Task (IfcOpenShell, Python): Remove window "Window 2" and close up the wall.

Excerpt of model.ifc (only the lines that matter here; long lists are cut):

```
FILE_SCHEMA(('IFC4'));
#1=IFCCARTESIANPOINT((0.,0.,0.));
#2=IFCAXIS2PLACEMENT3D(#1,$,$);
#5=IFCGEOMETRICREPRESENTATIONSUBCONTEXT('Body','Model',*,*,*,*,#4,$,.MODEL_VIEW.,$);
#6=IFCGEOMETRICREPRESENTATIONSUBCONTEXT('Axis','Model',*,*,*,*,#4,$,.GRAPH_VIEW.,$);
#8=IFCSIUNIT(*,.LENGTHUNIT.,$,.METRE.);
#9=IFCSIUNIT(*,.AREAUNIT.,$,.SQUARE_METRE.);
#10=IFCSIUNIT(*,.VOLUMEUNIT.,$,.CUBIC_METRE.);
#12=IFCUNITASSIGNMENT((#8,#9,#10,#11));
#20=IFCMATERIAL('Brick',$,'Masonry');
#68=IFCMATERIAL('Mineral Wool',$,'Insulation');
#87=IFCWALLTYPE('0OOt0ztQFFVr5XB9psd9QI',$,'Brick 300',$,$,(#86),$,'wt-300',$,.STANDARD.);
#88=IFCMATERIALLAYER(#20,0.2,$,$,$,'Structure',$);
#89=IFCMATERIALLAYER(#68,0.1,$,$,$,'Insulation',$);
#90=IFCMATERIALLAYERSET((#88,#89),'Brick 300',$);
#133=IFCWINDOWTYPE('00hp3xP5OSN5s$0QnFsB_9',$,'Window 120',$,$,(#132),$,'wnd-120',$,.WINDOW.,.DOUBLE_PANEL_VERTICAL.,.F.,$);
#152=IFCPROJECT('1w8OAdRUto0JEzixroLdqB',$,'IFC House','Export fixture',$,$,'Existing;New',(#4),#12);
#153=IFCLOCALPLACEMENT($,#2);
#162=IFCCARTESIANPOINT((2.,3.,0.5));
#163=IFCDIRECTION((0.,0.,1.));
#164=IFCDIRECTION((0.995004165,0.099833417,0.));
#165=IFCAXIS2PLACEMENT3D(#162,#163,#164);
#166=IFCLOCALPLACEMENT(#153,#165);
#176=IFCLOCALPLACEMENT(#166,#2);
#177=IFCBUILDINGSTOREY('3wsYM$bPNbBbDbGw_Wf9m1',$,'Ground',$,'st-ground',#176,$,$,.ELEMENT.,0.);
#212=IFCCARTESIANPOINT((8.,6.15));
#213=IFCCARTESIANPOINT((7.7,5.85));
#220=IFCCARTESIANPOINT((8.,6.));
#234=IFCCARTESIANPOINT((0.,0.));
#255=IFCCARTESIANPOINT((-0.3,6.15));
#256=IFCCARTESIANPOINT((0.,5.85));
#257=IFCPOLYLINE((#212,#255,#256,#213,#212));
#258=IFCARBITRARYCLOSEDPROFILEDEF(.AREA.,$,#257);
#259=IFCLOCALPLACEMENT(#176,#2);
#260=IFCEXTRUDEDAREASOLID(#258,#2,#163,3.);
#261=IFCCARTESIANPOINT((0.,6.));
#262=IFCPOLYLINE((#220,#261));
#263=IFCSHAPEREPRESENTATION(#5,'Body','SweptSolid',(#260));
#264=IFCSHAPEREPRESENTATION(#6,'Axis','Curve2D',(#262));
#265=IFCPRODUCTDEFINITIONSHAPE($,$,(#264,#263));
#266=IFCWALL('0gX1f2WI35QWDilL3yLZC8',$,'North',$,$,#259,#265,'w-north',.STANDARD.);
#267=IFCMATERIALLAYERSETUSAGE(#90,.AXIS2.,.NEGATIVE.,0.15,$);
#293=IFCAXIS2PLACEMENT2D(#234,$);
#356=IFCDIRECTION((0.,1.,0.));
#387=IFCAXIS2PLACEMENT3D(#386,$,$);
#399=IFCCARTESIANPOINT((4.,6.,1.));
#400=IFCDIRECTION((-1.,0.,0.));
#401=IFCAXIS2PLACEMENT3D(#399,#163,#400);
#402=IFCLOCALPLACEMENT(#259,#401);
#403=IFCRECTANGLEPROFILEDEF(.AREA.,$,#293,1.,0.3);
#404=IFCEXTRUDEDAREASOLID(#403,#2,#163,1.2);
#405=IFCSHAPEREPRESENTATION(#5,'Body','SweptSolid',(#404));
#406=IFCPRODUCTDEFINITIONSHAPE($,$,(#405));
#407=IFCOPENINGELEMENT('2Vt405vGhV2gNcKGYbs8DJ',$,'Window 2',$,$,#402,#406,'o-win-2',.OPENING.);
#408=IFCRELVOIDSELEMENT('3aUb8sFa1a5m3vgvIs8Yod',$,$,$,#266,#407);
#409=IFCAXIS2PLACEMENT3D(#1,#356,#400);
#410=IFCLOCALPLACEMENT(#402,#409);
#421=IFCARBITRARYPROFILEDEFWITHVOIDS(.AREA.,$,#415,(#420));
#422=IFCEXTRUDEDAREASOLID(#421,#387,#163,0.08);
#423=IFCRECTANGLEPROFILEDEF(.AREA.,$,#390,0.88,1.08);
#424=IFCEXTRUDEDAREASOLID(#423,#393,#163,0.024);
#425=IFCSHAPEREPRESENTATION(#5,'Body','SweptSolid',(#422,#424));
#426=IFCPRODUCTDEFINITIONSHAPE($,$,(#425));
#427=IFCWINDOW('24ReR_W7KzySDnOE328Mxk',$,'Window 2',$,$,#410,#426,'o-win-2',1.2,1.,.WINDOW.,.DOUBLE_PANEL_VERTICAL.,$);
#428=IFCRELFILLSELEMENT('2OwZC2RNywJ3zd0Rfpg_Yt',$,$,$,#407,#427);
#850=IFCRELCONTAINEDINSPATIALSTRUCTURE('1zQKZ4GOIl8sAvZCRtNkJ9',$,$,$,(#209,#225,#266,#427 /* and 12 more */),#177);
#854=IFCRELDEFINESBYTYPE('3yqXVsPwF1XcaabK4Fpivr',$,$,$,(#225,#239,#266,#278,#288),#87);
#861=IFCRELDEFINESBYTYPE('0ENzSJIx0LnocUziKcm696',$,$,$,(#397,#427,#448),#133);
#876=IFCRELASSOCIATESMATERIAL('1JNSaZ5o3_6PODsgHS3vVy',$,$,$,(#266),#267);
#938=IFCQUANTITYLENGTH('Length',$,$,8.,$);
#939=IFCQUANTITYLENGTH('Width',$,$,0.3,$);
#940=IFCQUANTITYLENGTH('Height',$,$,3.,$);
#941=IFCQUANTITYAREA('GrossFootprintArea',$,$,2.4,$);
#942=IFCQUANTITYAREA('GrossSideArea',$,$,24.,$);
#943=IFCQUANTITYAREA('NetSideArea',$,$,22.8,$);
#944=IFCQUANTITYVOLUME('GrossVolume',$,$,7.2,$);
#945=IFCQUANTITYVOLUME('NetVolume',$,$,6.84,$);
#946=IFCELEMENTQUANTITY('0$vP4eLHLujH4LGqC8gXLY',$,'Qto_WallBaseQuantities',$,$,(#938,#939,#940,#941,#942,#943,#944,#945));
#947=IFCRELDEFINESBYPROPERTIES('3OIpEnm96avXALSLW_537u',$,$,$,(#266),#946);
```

```python
import ifcopenshell
import ifcopenshell.api.feature
import ifcopenshell.api.pset
import ifcopenshell.api.root
import ifcopenshell.geom
import ifcopenshell.util.element
import ifcopenshell.util.shape
import ifcopenshell.util.unit

model = ifcopenshell.open("model.ifc")
area_scale = ifcopenshell.util.unit.calculate_unit_scale(model, "AREAUNIT")
volume_scale = ifcopenshell.util.unit.calculate_unit_scale(model, "VOLUMEUNIT")
settings = ifcopenshell.geom.settings()


def volume(element):
    """Net volume in cubic metres, openings subtracted."""
    shape = ifcopenshell.geom.create_shape(settings, element)
    return ifcopenshell.util.shape.get_volume(shape.geometry)


window = model.by_guid("24ReR_W7KzySDnOE328Mxk")
opening = window.FillsVoids[0].RelatingOpeningElement
wall = opening.VoidsElements[0].RelatingBuildingElement
before = volume(wall)

ifcopenshell.api.root.remove_product(model, product=window)
ifcopenshell.api.feature.remove_feature(model, feature=opening)

after = volume(wall)
thickness = 0.3  # wall thickness in metres

# Update the wall's stored quantities.
qto = model.by_id(ifcopenshell.util.element.get_pset(wall, "Qto_WallBaseQuantities", should_inherit=False)["id"])
ifcopenshell.api.pset.edit_qto(model, qto=qto, properties={
    "NetSideArea": after / thickness / area_scale,
    "NetVolume": after / volume_scale,
})

print(f"wall volume {before:.3f} -> {after:.3f} m3")

model.write("model_updated.ifc")
```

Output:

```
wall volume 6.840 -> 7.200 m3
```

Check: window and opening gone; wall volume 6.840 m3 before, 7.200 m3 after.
